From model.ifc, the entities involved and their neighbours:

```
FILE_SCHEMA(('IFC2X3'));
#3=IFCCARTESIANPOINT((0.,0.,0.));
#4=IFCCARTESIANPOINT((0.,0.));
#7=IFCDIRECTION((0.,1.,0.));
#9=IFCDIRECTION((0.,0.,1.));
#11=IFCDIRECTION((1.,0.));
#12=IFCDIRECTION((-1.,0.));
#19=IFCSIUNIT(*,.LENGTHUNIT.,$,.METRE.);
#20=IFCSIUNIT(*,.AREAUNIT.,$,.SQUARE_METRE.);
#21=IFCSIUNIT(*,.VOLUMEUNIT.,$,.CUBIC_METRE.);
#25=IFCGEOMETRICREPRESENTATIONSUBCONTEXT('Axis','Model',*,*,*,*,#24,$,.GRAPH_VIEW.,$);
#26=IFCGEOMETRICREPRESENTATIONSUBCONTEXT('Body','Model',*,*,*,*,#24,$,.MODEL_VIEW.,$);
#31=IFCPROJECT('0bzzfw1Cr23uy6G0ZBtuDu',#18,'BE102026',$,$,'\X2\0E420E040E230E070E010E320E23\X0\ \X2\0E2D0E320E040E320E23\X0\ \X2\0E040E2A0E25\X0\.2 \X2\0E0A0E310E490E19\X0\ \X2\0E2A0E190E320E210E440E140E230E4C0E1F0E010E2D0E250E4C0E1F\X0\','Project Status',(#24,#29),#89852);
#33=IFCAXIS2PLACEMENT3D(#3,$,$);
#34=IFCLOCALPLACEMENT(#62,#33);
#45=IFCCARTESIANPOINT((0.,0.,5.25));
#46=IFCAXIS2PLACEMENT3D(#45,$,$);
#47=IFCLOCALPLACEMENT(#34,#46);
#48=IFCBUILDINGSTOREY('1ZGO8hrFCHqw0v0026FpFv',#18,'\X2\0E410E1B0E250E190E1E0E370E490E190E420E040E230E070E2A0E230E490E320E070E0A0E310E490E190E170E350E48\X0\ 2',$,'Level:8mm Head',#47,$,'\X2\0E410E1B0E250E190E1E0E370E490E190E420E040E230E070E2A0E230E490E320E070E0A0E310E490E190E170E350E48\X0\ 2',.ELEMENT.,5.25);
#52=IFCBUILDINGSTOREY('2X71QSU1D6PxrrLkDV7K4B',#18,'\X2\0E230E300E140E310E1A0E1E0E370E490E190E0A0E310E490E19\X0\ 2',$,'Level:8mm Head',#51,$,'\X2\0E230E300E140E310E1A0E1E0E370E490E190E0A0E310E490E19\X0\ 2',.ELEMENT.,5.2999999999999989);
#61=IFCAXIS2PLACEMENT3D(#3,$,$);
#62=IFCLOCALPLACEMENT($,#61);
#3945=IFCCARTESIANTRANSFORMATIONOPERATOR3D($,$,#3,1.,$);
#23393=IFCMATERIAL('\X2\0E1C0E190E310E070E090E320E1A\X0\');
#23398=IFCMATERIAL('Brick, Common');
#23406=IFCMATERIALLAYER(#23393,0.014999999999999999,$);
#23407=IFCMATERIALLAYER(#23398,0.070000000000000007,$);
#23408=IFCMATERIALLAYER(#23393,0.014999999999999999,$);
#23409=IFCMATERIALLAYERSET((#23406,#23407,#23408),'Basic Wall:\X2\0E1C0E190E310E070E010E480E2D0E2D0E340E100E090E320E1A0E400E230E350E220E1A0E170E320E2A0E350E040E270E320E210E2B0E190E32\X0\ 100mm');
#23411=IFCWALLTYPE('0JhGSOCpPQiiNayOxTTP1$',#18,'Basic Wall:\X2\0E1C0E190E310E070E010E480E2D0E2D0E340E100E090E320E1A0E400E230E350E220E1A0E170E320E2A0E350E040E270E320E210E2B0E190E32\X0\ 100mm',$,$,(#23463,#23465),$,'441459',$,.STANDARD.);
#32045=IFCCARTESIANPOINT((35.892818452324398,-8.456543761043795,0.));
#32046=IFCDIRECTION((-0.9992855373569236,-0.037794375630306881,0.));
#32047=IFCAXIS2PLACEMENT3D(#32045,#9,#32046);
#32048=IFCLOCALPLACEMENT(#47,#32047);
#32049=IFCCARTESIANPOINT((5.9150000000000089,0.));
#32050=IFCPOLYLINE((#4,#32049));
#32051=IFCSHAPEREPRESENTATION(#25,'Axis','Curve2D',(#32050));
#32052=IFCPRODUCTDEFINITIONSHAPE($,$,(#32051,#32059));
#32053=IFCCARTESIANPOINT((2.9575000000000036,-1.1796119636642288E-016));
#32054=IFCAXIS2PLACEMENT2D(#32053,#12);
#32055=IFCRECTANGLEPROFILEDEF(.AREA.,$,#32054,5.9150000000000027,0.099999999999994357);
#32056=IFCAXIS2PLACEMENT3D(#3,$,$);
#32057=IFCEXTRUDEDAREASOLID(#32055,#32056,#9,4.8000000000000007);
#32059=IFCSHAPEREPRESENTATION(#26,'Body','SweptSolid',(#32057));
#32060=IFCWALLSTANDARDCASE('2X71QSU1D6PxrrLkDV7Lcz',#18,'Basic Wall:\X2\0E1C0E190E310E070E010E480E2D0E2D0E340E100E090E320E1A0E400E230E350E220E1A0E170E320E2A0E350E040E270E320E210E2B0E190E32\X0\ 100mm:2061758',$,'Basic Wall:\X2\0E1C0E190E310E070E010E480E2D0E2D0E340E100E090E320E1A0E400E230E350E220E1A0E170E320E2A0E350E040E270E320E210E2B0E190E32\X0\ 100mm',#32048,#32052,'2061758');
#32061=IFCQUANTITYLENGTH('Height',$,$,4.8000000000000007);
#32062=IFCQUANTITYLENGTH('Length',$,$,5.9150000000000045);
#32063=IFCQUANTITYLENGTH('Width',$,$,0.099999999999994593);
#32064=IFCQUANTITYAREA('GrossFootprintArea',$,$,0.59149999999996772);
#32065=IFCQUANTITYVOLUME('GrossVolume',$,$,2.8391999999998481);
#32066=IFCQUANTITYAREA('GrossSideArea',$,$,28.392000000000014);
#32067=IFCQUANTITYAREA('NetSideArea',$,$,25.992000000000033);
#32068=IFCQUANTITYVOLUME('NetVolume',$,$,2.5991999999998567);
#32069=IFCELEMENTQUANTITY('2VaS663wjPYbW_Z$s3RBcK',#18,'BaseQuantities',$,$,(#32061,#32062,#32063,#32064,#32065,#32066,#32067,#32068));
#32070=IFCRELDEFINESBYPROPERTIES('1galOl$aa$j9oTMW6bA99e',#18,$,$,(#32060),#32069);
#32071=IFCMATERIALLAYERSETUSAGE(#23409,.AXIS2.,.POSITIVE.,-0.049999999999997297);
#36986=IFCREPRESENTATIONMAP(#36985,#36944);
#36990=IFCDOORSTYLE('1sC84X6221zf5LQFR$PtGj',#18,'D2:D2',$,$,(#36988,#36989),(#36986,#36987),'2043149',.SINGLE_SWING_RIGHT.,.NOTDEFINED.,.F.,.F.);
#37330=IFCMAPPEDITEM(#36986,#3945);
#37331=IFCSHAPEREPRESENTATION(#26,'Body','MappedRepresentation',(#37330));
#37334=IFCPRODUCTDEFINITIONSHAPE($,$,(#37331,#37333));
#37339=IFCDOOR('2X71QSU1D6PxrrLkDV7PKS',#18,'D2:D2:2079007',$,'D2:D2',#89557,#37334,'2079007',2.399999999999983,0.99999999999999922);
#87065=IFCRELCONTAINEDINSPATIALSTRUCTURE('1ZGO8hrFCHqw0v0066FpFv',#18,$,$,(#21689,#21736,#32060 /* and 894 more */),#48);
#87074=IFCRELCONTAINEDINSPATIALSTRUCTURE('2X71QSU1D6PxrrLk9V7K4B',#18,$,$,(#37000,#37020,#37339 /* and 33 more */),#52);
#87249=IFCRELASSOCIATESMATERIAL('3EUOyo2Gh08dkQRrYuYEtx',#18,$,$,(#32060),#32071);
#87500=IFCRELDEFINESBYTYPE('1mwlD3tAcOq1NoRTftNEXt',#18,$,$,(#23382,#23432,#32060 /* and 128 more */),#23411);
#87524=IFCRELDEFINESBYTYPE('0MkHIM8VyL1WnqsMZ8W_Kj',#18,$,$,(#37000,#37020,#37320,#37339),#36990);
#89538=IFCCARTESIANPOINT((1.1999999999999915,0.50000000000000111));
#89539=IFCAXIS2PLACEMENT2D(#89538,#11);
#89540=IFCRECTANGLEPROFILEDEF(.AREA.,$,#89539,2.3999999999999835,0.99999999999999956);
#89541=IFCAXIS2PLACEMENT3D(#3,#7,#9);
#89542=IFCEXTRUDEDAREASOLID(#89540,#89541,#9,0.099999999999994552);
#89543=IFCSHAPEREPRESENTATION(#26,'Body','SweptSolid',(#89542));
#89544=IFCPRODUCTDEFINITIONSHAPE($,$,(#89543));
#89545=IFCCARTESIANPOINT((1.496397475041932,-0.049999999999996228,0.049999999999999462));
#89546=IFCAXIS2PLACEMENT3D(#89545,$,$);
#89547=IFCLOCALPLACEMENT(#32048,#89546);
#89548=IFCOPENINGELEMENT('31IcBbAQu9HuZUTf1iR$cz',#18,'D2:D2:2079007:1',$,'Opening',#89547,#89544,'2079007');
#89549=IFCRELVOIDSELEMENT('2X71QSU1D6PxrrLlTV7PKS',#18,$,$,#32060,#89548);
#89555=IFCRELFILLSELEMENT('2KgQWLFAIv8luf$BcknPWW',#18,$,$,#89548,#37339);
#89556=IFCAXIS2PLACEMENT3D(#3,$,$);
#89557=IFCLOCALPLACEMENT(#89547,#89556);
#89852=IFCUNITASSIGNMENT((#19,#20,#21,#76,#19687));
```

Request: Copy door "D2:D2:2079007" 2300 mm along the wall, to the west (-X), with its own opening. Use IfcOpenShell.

```python
import ifcopenshell
import ifcopenshell.api.feature
import ifcopenshell.api.geometry
import ifcopenshell.api.pset
import ifcopenshell.api.root
import ifcopenshell.geom
import ifcopenshell.util.element
import ifcopenshell.util.placement
import ifcopenshell.util.shape
import ifcopenshell.util.unit

model = ifcopenshell.open("model.ifc")
area_scale = ifcopenshell.util.unit.calculate_unit_scale(model, "AREAUNIT")
volume_scale = ifcopenshell.util.unit.calculate_unit_scale(model, "VOLUMEUNIT")
settings = ifcopenshell.geom.settings()


def volume(element):
    """Net volume in cubic metres, openings subtracted."""
    shape = ifcopenshell.geom.create_shape(settings, element)
    return ifcopenshell.util.shape.get_volume(shape.geometry)


def reuse_history(source, copy):
    """copy_class also copies each property set's owner history, people and application; keep the originals."""
    for rel in copy.IsDefinedBy:
        if rel.is_a("IfcRelDefinesByProperties") and (history := rel.RelatingPropertyDefinition.OwnerHistory):
            rel.RelatingPropertyDefinition.OwnerHistory = source.OwnerHistory
            ifcopenshell.util.element.remove_deep2(model, history)


door = model.by_guid("2X71QSU1D6PxrrLkDV7PKS")
opening = door.FillsVoids[0].RelatingOpeningElement
wall = opening.VoidsElements[0].RelatingBuildingElement
before = volume(wall)
shift = ifcopenshell.util.placement.get_local_placement(wall.ObjectPlacement)[:3, 0] * 2.3

# copy_class copies the void relationship, type, container and properties, but no geometry.
new_opening = ifcopenshell.api.root.copy_class(model, product=opening)
new_opening.Representation = ifcopenshell.util.element.copy_deep(
    model, opening.Representation, exclude=["IfcGeometricRepresentationContext", "IfcRepresentationMap"]
)
new_opening.Name = "D2:D2"
new_opening.Tag = None
reuse_history(opening, new_opening)
new_door = ifcopenshell.api.root.copy_class(model, product=door)
new_door.Representation = ifcopenshell.util.element.copy_deep(
    model, door.Representation, exclude=["IfcGeometricRepresentationContext", "IfcRepresentationMap"]
)
new_door.Name = "D2:D2"
new_door.Tag = None
reuse_history(door, new_door)
fills = ifcopenshell.api.feature.add_filling(model, opening=new_opening, element=new_door)
fills.OwnerHistory = new_door.OwnerHistory  # required in IFC2X3

for old, new in ((opening, new_opening), (door, new_door)):
    matrix = ifcopenshell.util.placement.get_local_placement(old.ObjectPlacement)
    matrix[:3, 3] += shift
    ifcopenshell.api.geometry.edit_object_placement(model, product=new, matrix=matrix, is_si=False)

after = volume(wall)
thickness = 0.1  # wall thickness in metres

# Update the wall's stored quantities.
qto = model.by_id(ifcopenshell.util.element.get_pset(wall, "BaseQuantities", should_inherit=False)["id"])
ifcopenshell.api.pset.edit_qto(model, qto=qto, properties={
    "NetSideArea": after / thickness / area_scale,
    "NetVolume": after / volume_scale,
})

print(f"wall volume {before:.3f} -> {after:.3f} m3")

model.write("model-out.ifc")
```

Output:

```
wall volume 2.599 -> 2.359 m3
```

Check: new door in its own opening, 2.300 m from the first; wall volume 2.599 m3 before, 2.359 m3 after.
